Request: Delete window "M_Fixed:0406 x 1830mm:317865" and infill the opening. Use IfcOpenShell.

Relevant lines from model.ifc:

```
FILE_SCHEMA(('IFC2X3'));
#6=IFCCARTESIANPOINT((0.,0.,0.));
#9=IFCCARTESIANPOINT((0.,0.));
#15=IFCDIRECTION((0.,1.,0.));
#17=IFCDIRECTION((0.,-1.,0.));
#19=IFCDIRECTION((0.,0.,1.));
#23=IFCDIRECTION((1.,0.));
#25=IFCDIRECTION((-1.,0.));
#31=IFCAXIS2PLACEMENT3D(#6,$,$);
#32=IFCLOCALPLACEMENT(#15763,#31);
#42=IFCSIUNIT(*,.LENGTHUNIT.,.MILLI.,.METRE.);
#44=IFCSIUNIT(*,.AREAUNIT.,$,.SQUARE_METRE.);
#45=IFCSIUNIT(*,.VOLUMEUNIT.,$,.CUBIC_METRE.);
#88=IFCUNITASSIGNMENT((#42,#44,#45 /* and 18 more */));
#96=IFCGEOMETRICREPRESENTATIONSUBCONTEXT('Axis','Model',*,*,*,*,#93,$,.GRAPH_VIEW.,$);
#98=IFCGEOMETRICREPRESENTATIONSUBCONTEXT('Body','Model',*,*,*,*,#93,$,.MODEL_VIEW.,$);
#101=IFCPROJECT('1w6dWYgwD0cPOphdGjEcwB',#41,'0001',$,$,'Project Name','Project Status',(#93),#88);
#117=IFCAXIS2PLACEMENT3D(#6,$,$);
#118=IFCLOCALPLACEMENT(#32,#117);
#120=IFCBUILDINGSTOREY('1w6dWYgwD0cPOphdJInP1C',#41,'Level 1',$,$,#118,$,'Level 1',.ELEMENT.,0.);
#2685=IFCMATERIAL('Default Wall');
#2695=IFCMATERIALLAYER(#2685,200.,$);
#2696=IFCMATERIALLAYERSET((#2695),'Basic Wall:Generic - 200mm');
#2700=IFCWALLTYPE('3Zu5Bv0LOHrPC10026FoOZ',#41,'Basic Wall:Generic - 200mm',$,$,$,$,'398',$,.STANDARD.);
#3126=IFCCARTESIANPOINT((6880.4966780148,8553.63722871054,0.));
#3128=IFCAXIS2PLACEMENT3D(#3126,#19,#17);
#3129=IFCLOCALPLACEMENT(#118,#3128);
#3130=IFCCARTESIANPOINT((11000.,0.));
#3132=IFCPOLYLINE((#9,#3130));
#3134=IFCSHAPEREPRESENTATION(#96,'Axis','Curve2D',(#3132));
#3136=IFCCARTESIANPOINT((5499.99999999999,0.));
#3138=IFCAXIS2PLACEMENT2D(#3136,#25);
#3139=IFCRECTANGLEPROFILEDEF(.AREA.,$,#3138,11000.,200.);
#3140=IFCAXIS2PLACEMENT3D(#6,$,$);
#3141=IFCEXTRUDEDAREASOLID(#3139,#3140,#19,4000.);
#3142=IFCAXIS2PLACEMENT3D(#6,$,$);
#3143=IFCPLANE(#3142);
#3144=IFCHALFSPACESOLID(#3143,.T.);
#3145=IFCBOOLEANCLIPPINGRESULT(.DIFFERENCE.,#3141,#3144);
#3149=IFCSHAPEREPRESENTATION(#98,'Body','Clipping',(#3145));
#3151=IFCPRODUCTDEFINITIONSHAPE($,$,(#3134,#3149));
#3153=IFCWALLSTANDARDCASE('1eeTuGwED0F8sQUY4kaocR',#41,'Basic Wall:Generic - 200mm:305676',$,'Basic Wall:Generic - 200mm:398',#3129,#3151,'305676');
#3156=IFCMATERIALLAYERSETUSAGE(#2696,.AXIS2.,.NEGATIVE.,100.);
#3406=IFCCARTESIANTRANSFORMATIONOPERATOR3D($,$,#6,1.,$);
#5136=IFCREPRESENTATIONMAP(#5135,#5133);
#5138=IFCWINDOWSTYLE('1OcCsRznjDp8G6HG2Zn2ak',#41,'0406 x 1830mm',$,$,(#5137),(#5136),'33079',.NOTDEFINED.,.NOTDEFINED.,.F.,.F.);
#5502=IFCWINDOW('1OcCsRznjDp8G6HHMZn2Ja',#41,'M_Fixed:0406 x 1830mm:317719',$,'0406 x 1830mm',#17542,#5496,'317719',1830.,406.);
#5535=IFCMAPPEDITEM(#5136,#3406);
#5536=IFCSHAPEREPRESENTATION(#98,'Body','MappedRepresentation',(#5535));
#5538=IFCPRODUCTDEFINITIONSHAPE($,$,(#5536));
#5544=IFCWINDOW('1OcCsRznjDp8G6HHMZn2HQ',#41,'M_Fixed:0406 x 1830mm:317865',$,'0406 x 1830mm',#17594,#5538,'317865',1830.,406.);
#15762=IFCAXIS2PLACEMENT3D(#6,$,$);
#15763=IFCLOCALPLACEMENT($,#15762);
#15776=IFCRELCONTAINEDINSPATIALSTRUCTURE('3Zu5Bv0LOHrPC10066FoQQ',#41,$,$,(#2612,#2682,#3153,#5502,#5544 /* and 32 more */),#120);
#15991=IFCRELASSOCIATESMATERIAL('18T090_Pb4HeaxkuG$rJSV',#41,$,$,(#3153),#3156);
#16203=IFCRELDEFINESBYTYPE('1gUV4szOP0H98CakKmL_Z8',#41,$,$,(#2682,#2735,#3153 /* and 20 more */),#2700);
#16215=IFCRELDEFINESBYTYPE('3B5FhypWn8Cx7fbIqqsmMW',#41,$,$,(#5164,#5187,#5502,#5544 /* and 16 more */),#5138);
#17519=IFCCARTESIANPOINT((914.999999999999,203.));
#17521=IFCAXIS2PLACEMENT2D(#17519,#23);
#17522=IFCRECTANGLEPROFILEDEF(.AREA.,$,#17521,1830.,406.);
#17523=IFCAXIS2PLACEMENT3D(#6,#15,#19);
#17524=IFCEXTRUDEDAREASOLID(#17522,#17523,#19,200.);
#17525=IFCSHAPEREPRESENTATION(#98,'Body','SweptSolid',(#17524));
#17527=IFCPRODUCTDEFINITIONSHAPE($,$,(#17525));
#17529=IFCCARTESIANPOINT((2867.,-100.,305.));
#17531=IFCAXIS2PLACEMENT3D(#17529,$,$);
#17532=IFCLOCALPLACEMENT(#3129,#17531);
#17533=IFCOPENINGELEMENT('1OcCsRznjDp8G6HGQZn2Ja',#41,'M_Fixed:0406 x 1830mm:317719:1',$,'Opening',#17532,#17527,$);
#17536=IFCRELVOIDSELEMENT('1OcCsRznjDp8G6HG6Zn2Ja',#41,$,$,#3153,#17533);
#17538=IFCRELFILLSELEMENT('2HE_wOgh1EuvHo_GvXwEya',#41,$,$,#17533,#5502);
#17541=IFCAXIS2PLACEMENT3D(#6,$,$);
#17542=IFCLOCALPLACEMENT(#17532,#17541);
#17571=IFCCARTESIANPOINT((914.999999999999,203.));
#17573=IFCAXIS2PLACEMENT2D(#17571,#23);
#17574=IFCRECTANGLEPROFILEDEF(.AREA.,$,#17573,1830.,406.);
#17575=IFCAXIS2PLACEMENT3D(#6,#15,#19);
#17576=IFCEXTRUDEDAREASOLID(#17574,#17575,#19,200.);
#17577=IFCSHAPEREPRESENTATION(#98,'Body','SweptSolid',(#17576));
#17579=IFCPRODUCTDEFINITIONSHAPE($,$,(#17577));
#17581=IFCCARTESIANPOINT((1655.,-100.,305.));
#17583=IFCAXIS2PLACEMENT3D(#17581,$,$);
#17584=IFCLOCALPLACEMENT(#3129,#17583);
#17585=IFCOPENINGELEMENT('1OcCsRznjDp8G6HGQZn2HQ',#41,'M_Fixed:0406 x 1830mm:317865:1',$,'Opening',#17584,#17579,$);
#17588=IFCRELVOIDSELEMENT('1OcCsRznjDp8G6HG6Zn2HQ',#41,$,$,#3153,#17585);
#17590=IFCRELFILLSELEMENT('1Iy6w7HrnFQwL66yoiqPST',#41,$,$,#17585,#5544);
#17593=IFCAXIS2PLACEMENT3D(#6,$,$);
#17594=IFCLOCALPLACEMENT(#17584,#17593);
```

```python
import ifcopenshell
import ifcopenshell.api.feature
import ifcopenshell.api.root
import ifcopenshell.geom
import ifcopenshell.util.shape

model = ifcopenshell.open("model.ifc")
settings = ifcopenshell.geom.settings()


def volume(element):
    """Net volume in cubic metres, openings subtracted."""
    shape = ifcopenshell.geom.create_shape(settings, element)
    return ifcopenshell.util.shape.get_volume(shape.geometry)


window = model.by_id(5544)
opening = window.FillsVoids[0].RelatingOpeningElement
wall = opening.VoidsElements[0].RelatingBuildingElement
before = volume(wall)

ifcopenshell.api.root.remove_product(model, product=window)
ifcopenshell.api.feature.remove_feature(model, feature=opening)

after = volume(wall)

print(f"wall volume {before:.3f} -> {after:.3f} m3")

model.write("model_updated.ifc")
```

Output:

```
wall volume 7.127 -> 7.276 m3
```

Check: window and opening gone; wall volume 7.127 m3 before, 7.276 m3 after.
